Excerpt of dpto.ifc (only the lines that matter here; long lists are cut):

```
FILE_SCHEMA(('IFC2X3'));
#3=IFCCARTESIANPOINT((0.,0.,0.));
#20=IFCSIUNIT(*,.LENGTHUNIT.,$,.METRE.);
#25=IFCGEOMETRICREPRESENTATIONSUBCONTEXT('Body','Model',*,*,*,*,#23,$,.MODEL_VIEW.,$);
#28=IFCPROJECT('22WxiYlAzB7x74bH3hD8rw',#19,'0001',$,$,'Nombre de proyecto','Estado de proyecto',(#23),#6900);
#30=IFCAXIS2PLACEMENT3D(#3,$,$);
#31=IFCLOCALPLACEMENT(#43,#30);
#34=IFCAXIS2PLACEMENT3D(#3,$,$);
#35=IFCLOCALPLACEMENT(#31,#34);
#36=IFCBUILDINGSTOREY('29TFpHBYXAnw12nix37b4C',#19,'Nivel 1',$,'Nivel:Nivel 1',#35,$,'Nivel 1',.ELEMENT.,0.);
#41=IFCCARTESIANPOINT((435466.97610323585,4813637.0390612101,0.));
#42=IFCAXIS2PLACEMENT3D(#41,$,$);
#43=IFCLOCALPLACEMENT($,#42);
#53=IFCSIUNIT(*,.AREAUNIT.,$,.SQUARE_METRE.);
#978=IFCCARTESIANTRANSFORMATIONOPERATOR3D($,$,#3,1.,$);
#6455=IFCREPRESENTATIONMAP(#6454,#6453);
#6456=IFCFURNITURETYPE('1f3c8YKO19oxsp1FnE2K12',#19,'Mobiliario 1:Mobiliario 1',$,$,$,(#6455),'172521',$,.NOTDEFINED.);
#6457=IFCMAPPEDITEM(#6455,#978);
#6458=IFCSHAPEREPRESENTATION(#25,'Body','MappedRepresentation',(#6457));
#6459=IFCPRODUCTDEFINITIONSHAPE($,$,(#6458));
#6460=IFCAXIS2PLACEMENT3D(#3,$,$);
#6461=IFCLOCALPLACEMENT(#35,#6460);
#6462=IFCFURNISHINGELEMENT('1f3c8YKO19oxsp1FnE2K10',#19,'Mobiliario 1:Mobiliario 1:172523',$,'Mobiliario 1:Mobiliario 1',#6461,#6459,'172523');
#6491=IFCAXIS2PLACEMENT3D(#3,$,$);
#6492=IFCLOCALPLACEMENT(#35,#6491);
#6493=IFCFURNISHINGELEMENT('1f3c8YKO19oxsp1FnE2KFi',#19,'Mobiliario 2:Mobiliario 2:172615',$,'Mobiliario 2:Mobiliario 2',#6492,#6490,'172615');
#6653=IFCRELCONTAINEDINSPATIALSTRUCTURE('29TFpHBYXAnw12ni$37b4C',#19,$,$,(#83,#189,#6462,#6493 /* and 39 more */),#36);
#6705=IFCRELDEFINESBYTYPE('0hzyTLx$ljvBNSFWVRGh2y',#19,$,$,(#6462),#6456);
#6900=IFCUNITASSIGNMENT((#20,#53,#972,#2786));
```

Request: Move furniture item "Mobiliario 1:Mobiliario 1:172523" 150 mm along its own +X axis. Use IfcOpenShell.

```python
import ifcopenshell
import ifcopenshell.api.geometry
import ifcopenshell.util.placement

model = ifcopenshell.open("dpto.ifc")

item = model.by_id(6462)
matrix = ifcopenshell.util.placement.get_local_placement(item.ObjectPlacement)
matrix[:3, 3] += matrix[:3, 0] * 0.15
ifcopenshell.api.geometry.edit_object_placement(model, product=item, matrix=matrix, is_si=False)

print(ifcopenshell.util.placement.get_local_placement(item.ObjectPlacement).round(3) + 0.0)

model.write("dpto_updated.ifc")
```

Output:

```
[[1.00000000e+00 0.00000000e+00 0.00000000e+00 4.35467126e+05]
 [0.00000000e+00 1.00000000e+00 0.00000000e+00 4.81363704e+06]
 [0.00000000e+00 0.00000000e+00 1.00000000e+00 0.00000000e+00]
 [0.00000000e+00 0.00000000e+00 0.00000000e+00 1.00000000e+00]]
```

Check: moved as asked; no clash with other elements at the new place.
